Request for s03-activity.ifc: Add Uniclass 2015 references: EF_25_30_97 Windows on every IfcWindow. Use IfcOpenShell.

First a look at what the model holds.

```python
import ifcopenshell

model = ifcopenshell.open("s03-activity.ifc")
print(model.schema)
print("classifications:", [c.Name for c in model.by_type("IfcClassification")])
for ifc_class in ("IfcDoor", "IfcRoof", "IfcStair", "IfcWall", "IfcWindow"):
    print(ifc_class, len(model.by_type(ifc_class)))
```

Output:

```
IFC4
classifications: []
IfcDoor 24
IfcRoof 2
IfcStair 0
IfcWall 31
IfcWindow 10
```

```python
import ifcopenshell
import ifcopenshell.api.classification

model = ifcopenshell.open("s03-activity.ifc")

system = ifcopenshell.api.classification.add_classification(model, classification="Uniclass 2015")

codes = {
    "IfcWindow": ("EF_25_30_97", "Windows"),
}
for ifc_class, (code, name) in codes.items():
    products = model.by_type(ifc_class)
    ifcopenshell.api.classification.add_reference(
        model, products=products, classification=system, identification=code, name=name
    )
    print(code, len(products))

model.write("s03-activity_updated.ifc")
```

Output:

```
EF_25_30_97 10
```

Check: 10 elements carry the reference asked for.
